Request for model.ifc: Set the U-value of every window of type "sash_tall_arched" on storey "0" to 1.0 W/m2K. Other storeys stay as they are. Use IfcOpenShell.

First a look at what the model holds.

```python
import ifcopenshell
import ifcopenshell.util.element

model = ifcopenshell.open("model.ifc")
print(model.schema)
storey = next(s for s in model.by_type("IfcBuildingStorey") if s.Name == "0")
windows = [e for e in ifcopenshell.util.element.get_decomposition(storey) if e.is_a("IfcWindow")]
seen = {}
for e in windows:
    element_type = ifcopenshell.util.element.get_type(e)
    key = (element_type.Name if element_type != e and element_type else None, ifcopenshell.util.element.get_pset(e, "Pset_WindowCommon", "ThermalTransmittance"))
    seen[key] = seen.get(key, 0) + 1
for (name, value), count in sorted(seen.items(), key=str):
    print(count, "x", name, "|", value)
```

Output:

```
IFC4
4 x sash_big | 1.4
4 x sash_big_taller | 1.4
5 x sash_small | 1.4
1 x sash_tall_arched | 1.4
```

```python
import ifcopenshell
import ifcopenshell.api.pset
import ifcopenshell.util.element

model = ifcopenshell.open("model.ifc")

storey = next(s for s in model.by_type("IfcBuildingStorey") if s.Name == "0")
windows = [e for e in ifcopenshell.util.element.get_decomposition(storey) if e.is_a("IfcWindow")]

count = 0
for e in windows:
    element_type = ifcopenshell.util.element.get_type(e)
    if element_type in (None, e) or element_type.Name != "sash_tall_arched":
        continue
    # add_pset returns the element's existing set when there is one.
    pset = ifcopenshell.api.pset.add_pset(model, product=e, name="Pset_WindowCommon")
    ifcopenshell.api.pset.edit_pset(model, pset=pset, properties={"ThermalTransmittance": 1.0})
    count += 1

print(count, "windows updated")

model.write("model_rev.ifc")
```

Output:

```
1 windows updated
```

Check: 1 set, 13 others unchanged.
